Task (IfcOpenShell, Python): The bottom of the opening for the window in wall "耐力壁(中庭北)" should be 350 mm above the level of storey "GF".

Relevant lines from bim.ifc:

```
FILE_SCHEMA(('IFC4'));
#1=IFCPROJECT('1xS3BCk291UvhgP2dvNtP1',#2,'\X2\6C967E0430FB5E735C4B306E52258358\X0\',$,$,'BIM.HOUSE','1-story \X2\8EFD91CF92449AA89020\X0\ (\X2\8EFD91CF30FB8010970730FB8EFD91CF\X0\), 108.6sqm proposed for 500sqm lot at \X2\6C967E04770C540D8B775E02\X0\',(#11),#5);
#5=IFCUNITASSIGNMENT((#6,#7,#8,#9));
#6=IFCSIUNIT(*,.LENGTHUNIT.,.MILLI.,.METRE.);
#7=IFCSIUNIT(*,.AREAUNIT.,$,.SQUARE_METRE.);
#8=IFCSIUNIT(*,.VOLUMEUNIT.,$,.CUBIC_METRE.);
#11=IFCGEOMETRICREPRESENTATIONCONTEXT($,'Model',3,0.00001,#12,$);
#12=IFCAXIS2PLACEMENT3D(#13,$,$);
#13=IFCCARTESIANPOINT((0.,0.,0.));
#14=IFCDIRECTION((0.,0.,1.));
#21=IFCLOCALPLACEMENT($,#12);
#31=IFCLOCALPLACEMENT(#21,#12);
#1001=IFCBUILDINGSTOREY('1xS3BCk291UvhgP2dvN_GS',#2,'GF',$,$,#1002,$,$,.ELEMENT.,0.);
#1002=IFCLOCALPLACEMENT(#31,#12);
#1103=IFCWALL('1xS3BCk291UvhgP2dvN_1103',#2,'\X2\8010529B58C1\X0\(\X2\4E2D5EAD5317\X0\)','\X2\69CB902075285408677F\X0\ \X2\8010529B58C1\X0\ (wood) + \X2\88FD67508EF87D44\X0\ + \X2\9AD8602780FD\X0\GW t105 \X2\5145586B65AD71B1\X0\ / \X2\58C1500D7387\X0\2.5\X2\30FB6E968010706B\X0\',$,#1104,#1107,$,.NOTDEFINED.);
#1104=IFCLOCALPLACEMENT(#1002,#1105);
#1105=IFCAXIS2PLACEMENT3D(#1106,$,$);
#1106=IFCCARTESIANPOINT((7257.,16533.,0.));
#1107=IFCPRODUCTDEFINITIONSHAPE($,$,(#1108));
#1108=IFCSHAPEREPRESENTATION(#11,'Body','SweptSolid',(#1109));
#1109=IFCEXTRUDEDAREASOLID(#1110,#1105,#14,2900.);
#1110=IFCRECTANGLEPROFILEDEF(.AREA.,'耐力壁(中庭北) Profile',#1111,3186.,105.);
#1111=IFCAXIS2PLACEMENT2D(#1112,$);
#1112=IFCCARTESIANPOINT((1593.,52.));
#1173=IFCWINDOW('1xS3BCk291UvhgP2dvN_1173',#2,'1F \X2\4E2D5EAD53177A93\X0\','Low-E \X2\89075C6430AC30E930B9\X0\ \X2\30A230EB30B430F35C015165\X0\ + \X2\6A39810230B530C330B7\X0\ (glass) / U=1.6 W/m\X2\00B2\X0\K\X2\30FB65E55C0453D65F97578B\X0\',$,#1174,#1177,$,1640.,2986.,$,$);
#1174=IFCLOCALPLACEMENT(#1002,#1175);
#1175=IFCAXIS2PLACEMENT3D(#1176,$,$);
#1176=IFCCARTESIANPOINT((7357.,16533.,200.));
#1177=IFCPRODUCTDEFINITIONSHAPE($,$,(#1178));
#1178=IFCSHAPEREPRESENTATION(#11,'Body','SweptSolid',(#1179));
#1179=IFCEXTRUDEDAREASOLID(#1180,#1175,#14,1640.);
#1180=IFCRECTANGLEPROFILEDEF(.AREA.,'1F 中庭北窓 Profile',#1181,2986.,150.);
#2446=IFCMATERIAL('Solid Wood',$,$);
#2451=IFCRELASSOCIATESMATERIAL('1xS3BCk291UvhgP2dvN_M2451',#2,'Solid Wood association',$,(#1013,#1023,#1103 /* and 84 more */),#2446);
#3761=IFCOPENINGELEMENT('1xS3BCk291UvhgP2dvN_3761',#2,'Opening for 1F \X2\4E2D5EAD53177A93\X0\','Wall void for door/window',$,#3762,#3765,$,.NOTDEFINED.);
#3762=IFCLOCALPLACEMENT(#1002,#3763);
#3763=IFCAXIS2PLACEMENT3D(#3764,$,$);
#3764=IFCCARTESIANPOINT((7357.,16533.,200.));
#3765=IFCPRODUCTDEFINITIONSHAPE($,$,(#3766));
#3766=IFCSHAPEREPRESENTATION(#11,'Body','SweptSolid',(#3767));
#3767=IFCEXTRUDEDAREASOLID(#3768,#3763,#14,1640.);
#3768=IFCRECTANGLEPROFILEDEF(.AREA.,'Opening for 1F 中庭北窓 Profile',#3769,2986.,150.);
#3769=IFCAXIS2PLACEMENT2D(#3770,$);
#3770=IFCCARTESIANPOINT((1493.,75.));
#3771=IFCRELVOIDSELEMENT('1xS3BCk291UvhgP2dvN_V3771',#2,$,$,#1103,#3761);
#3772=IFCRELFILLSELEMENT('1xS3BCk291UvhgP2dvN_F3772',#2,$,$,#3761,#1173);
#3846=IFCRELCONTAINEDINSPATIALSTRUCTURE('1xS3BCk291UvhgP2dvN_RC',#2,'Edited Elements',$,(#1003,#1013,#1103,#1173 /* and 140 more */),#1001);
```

```python
import numpy as np
import ifcopenshell
import ifcopenshell.api.geometry
import ifcopenshell.geom
import ifcopenshell.util.element
import ifcopenshell.util.placement
import ifcopenshell.util.shape
import ifcopenshell.util.unit

model = ifcopenshell.open("bim.ifc")
unit_scale = ifcopenshell.util.unit.calculate_unit_scale(model)

window = model.by_id(1173)
opening = window.FillsVoids[0].RelatingOpeningElement
storey = ifcopenshell.util.element.get_container(window, ifc_class="IfcBuildingStorey")
level = ifcopenshell.util.placement.get_local_placement(storey.ObjectPlacement)[2, 3]

# The opening's origin need not be at the sill, so measure its lowest point.
shape = ifcopenshell.geom.create_shape(ifcopenshell.geom.settings(), opening)
bottom = ifcopenshell.util.shape.get_shape_bottom_elevation(shape, shape.geometry) / unit_scale
dz = level + 0.35 / unit_scale - bottom

shift = np.array([0.0, 0.0, dz])
# The window is not placed relative to its opening, so move both.
for product in (opening, window):
    matrix = ifcopenshell.util.placement.get_local_placement(product.ObjectPlacement)
    matrix[:3, 3] += shift
    ifcopenshell.api.geometry.edit_object_placement(model, product=product, matrix=matrix, is_si=False)

print(f"moved by {dz * unit_scale:+.3f} m")

model.write("bim_v2.ifc")
```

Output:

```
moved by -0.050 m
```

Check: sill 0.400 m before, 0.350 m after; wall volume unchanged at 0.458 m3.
